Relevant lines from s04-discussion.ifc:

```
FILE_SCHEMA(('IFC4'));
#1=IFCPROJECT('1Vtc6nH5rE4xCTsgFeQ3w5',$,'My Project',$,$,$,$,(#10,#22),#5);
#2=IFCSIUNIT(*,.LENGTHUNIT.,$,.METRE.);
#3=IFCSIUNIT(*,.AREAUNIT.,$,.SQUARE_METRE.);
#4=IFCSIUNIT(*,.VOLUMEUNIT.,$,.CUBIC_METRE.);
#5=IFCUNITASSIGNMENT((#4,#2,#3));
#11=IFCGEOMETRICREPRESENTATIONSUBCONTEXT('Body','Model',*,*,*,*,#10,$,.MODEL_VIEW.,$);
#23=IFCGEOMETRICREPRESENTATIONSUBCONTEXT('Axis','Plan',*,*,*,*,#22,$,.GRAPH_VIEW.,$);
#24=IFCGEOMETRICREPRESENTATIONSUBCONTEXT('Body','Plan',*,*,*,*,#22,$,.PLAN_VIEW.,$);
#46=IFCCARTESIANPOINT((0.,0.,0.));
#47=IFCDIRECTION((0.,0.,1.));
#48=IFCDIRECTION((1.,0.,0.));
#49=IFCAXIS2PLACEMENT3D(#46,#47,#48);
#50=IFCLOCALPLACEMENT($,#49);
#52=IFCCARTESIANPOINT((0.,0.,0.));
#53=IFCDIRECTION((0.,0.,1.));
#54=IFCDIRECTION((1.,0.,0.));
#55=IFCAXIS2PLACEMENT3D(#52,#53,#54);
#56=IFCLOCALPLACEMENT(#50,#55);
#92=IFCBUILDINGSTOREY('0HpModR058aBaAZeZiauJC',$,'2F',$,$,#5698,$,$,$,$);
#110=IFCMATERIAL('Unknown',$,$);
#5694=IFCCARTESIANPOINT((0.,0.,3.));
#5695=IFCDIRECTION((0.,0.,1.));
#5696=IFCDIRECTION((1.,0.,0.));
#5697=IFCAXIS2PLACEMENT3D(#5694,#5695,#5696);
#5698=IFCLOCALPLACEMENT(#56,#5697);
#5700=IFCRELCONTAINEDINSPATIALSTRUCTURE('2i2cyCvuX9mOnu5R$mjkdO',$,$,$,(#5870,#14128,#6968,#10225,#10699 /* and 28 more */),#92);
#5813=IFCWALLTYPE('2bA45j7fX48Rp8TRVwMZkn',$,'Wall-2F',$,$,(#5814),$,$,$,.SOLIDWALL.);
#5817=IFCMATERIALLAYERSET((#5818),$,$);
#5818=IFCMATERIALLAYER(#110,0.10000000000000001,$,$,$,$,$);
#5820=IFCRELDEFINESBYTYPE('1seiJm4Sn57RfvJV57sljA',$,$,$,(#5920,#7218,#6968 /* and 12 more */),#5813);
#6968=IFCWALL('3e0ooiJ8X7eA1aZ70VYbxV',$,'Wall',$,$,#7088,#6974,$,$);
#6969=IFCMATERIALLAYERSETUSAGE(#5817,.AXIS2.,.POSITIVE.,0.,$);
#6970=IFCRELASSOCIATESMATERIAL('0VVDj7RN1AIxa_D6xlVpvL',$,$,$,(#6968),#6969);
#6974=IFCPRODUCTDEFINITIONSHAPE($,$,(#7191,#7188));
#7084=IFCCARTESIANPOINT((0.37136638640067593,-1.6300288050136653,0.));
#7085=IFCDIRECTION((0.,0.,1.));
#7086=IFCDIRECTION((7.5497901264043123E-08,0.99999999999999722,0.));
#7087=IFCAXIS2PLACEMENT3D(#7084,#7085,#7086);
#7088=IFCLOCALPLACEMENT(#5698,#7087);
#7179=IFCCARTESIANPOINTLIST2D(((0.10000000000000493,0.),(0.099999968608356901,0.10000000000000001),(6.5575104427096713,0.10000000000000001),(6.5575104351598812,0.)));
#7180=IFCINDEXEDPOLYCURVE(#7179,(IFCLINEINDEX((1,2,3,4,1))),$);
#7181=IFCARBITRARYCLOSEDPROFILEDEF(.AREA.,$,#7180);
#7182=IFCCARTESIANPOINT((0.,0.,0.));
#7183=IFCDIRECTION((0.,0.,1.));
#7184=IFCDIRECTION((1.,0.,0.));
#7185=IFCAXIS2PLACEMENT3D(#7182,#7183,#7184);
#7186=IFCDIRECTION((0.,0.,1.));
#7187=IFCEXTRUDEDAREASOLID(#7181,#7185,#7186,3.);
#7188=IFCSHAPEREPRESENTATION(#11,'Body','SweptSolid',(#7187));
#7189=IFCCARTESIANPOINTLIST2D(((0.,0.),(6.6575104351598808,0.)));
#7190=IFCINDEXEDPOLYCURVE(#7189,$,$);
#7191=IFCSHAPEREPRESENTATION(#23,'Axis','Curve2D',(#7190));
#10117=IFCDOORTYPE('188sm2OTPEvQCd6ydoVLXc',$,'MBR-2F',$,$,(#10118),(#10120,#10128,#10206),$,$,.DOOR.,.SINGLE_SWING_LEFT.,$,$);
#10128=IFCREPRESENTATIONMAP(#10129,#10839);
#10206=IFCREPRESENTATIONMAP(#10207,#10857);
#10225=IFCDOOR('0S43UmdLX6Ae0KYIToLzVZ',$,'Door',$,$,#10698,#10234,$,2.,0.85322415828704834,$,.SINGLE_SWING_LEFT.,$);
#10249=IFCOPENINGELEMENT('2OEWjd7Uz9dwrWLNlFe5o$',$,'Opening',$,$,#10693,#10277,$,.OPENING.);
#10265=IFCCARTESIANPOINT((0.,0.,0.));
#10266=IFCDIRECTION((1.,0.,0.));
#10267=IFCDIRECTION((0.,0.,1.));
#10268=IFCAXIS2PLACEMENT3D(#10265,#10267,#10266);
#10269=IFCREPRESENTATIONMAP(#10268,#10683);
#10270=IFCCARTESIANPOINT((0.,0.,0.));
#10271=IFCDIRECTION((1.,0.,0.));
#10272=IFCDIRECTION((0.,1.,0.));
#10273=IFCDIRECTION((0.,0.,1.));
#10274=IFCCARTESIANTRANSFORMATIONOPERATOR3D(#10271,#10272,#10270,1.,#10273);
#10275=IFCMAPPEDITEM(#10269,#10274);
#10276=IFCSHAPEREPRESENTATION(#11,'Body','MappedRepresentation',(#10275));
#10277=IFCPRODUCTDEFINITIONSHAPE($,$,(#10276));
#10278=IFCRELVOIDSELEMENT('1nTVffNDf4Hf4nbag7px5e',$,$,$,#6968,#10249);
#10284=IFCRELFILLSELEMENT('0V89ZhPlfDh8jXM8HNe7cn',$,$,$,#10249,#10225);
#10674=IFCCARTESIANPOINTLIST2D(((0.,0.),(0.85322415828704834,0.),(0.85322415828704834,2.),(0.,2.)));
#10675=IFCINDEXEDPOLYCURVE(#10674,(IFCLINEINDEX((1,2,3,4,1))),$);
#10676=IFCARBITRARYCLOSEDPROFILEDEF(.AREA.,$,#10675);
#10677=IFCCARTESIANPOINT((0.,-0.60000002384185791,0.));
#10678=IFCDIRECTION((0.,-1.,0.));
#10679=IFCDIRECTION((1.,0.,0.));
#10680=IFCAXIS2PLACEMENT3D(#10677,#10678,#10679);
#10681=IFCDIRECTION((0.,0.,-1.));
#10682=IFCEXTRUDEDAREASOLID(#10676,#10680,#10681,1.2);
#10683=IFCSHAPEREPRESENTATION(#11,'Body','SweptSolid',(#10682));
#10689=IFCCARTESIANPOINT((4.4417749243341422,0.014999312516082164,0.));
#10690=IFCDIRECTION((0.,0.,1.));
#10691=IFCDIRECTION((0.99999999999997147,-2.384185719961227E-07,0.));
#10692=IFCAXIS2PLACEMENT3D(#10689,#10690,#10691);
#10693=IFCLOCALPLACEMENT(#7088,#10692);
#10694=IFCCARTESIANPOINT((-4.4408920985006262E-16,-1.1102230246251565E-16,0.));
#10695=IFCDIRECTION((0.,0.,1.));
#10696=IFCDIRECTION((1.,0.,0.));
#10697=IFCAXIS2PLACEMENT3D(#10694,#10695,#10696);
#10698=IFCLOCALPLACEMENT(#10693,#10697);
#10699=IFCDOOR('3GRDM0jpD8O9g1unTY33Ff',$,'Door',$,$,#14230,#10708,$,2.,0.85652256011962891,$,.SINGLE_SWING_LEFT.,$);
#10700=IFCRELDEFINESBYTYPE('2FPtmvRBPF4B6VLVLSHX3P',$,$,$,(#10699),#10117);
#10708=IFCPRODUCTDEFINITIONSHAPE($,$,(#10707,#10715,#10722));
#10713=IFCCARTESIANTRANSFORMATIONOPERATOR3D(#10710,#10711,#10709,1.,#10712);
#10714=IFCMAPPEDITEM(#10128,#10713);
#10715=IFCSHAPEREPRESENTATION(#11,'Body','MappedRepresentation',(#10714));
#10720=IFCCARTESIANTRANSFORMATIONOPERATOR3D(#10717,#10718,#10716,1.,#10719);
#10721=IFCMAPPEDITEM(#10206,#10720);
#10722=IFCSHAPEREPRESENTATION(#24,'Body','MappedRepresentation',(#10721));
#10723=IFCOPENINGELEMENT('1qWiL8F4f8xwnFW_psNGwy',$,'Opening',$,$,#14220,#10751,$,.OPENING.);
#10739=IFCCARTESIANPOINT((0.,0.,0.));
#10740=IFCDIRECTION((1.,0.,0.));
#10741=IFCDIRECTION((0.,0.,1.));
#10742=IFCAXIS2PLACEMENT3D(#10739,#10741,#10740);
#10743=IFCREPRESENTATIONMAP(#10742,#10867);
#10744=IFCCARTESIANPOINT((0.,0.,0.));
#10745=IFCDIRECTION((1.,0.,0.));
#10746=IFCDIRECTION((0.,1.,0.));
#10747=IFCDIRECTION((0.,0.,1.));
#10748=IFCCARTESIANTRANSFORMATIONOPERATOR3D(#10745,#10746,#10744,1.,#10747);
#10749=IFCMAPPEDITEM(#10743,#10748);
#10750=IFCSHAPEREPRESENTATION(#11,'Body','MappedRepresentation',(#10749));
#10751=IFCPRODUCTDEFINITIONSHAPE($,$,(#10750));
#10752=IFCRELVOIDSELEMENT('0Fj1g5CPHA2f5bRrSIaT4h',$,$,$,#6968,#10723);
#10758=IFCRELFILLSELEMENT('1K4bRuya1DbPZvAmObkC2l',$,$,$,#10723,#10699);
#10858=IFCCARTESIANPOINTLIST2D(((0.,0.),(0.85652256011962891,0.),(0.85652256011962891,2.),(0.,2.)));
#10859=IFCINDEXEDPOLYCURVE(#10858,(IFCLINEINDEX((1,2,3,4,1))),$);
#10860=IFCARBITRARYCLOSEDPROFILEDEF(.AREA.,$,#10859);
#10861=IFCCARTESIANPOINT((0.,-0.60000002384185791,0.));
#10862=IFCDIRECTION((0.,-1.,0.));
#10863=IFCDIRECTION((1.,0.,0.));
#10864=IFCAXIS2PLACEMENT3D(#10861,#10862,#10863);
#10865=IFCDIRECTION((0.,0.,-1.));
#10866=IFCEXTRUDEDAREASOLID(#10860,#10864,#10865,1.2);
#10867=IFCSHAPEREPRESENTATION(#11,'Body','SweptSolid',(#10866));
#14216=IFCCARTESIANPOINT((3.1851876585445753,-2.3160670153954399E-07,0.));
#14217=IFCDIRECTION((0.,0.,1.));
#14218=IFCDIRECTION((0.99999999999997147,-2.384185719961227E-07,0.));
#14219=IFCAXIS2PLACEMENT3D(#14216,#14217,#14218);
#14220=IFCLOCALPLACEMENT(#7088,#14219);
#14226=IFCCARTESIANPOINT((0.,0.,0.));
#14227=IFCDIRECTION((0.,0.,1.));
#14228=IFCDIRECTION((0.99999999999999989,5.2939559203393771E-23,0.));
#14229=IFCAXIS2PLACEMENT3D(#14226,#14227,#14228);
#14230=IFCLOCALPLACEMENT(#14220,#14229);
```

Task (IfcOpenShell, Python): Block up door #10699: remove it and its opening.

```python
import ifcopenshell
import ifcopenshell.api.feature
import ifcopenshell.api.root
import ifcopenshell.geom
import ifcopenshell.util.shape

model = ifcopenshell.open("s04-discussion.ifc")
settings = ifcopenshell.geom.settings()


def volume(element):
    """Net volume in cubic metres, openings subtracted."""
    shape = ifcopenshell.geom.create_shape(settings, element)
    return ifcopenshell.util.shape.get_volume(shape.geometry)


door = model.by_guid("3GRDM0jpD8O9g1unTY33Ff")
opening = door.FillsVoids[0].RelatingOpeningElement
wall = opening.VoidsElements[0].RelatingBuildingElement
before = volume(wall)

ifcopenshell.api.root.remove_product(model, product=door)
ifcopenshell.api.feature.remove_feature(model, feature=opening)

after = volume(wall)

print(f"wall volume {before:.3f} -> {after:.3f} m3")

model.write("s04-discussion_edited.ifc")
```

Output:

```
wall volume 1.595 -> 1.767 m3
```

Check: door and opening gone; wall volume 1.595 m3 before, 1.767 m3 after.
